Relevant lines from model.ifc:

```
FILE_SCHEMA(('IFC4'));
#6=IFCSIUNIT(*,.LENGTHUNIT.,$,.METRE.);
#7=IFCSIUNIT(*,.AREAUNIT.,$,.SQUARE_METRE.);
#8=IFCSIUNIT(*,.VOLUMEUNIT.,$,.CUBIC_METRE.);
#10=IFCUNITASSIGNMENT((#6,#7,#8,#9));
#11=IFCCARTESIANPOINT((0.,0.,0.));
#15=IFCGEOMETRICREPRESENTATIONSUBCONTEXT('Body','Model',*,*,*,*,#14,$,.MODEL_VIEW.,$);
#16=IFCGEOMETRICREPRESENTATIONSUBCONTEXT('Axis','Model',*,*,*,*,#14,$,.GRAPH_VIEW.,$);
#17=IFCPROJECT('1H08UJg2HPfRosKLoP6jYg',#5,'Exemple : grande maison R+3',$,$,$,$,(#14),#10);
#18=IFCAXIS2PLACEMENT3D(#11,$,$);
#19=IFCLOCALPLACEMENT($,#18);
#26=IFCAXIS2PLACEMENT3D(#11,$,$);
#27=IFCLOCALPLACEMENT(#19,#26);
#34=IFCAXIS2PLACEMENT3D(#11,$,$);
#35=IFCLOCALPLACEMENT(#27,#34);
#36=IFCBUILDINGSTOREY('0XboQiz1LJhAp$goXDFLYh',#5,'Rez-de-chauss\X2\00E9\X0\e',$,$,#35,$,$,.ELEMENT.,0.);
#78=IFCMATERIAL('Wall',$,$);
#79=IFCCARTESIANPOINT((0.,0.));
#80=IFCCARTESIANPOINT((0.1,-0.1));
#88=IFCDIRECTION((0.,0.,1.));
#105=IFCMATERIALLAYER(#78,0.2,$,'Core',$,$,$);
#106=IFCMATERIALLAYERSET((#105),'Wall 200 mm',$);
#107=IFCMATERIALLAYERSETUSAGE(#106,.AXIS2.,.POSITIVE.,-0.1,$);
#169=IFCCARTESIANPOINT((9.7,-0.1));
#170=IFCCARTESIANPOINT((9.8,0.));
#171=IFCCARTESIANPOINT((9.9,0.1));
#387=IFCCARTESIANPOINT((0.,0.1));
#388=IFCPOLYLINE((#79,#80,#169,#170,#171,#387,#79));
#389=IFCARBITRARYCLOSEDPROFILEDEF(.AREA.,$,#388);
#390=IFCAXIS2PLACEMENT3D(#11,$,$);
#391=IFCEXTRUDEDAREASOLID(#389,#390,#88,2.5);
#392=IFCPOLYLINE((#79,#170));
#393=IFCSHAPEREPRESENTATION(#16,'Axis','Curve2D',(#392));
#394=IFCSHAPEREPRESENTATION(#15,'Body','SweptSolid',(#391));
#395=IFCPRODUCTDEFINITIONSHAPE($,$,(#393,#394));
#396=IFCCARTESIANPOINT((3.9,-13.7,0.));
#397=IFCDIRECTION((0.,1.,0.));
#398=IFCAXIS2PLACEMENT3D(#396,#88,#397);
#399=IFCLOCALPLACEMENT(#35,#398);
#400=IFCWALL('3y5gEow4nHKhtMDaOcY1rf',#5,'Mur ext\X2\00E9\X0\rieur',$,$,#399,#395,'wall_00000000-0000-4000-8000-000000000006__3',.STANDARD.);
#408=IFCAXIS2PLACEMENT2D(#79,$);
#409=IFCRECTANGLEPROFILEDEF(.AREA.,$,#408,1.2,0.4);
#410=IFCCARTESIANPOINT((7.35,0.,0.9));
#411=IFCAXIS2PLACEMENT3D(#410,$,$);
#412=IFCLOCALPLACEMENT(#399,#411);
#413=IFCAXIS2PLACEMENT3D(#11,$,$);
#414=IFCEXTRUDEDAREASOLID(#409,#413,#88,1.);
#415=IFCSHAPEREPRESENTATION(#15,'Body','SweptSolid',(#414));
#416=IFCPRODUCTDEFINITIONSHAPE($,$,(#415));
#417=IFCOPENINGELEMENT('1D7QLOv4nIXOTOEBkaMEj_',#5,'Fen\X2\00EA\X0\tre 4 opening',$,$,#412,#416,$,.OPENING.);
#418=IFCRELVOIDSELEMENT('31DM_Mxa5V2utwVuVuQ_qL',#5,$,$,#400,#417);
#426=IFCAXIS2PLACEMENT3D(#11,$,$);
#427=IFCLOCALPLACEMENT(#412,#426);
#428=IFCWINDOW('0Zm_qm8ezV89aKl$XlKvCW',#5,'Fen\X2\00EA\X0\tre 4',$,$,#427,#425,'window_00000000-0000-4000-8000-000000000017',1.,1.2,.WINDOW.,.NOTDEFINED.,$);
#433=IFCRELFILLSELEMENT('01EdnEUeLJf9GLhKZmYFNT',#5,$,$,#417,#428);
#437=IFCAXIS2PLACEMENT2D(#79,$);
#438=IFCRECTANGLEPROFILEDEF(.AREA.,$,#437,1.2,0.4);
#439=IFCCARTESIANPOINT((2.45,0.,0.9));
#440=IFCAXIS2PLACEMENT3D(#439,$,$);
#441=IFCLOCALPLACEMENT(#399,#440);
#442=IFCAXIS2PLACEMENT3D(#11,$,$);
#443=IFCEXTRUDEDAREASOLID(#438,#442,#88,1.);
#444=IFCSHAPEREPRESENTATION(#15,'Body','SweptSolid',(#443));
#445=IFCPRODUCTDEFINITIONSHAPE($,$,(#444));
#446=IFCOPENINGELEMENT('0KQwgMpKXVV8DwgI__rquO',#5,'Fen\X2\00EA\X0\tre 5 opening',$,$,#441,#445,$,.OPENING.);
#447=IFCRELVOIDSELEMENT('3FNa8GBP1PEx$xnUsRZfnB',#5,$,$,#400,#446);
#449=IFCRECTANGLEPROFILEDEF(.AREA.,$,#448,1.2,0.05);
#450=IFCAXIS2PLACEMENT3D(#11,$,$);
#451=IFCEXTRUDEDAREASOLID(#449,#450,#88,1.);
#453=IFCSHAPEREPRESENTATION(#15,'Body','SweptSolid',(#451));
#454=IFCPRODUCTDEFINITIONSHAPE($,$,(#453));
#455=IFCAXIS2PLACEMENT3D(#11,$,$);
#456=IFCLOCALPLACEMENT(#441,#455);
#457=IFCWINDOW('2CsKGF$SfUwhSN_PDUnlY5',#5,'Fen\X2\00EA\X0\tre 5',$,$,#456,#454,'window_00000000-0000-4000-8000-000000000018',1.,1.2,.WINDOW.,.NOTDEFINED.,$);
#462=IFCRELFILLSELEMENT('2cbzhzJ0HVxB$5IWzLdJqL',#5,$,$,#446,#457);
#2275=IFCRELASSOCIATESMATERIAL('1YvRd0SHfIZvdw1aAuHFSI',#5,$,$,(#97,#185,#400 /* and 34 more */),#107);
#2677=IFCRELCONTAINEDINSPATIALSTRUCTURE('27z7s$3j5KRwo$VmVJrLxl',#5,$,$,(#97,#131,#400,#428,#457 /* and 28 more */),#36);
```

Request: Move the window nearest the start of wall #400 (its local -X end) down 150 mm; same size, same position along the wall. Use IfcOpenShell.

```python
import numpy as np
import ifcopenshell
import ifcopenshell.api.geometry
import ifcopenshell.util.placement
import ifcopenshell.util.unit

model = ifcopenshell.open("model.ifc")
unit_scale = ifcopenshell.util.unit.calculate_unit_scale(model)

window = model.by_guid("2CsKGF$SfUwhSN_PDUnlY5")
opening = window.FillsVoids[0].RelatingOpeningElement
dz = -0.15

shift = np.array([0.0, 0.0, dz])
# The window is placed relative to its opening, so it follows when the opening moves.
matrix = ifcopenshell.util.placement.get_local_placement(opening.ObjectPlacement)
matrix[:3, 3] += shift
ifcopenshell.api.geometry.edit_object_placement(
    model, product=opening, matrix=matrix, is_si=False, should_transform_children=True
)

print(f"moved by {dz * unit_scale:+.3f} m")

model.write("model_rev.ifc")
```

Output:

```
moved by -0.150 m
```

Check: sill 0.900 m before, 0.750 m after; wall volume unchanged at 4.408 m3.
